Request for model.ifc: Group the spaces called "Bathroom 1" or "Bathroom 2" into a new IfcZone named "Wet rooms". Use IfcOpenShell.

First a look at what the model holds.

```python
import ifcopenshell

model = ifcopenshell.open("model.ifc")
print(model.schema)
seen = {}
for space in model.by_type("IfcSpace"):
    seen[space.LongName] = seen.get(space.LongName, 0) + 1
for name, count in sorted(seen.items(), key=str):
    print(count, "x", name)
print("zones:", [z.Name for z in model.by_type("IfcZone")][:20])
```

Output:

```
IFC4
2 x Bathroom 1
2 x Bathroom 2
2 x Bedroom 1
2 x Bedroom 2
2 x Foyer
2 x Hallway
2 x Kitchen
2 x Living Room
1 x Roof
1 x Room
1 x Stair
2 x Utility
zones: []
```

```python
import ifcopenshell
import ifcopenshell.api.group
import ifcopenshell.api.root

model = ifcopenshell.open("model.ifc")

names = {"Bathroom 1", "Bathroom 2"}
spaces = [s for s in model.by_type("IfcSpace") if s.LongName in names]

zone = ifcopenshell.api.root.create_entity(model, ifc_class="IfcZone", name="Wet rooms")
ifcopenshell.api.group.assign_group(model, products=spaces, group=zone)
print(len(spaces), "spaces in", zone.Name)

model.write("model-out.ifc")
```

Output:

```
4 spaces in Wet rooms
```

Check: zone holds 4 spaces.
